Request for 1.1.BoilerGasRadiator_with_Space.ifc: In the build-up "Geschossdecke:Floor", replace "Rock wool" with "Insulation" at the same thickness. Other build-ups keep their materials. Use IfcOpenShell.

First a look at what the model holds.

```python
import ifcopenshell
import ifcopenshell.util.element

model = ifcopenshell.open("1.1.BoilerGasRadiator_with_Space.ifc")
print(model.schema)
for layer_set in model.by_type("IfcMaterialLayerSet"):
    if layer_set.LayerSetName == "Geschossdecke:Floor":
        for layer in layer_set.MaterialLayers:
            print(layer.id(), layer.Material and layer.Material.Name, layer.LayerThickness, sep=" | ")
        print(len(ifcopenshell.util.element.get_elements_by_material(model, layer_set)), "elements and types use it")
print(sorted(m.Name for m in model.by_type("IfcMaterial") if m.Name)[:60])
```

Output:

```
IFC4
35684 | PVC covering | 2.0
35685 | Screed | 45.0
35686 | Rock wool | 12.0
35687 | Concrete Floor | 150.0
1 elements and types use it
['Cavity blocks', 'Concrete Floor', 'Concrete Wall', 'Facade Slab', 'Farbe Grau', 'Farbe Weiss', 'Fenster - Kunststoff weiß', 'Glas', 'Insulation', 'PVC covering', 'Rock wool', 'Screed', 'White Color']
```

```python
import ifcopenshell
import ifcopenshell.api.material

model = ifcopenshell.open("1.1.BoilerGasRadiator_with_Space.ifc")

layer_set = next(s for s in model.by_type("IfcMaterialLayerSet") if s.LayerSetName == "Geschossdecke:Floor")
layer = next(l for l in layer_set.MaterialLayers if l.Material and l.Material.Name == "Rock wool")
material = next(m for m in model.by_type("IfcMaterial") if m.Name == "Insulation")

# Point this one layer at the other material; renaming the old one would change it everywhere.
ifcopenshell.api.material.edit_layer(model, layer=layer, attributes={}, material=material)

print([l.Material.Name if l.Material else None for l in layer_set.MaterialLayers])

model.write("1.1.BoilerGasRadiator_with_Space_v2.ifc")
```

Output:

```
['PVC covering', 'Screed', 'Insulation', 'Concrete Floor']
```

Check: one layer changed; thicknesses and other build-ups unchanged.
